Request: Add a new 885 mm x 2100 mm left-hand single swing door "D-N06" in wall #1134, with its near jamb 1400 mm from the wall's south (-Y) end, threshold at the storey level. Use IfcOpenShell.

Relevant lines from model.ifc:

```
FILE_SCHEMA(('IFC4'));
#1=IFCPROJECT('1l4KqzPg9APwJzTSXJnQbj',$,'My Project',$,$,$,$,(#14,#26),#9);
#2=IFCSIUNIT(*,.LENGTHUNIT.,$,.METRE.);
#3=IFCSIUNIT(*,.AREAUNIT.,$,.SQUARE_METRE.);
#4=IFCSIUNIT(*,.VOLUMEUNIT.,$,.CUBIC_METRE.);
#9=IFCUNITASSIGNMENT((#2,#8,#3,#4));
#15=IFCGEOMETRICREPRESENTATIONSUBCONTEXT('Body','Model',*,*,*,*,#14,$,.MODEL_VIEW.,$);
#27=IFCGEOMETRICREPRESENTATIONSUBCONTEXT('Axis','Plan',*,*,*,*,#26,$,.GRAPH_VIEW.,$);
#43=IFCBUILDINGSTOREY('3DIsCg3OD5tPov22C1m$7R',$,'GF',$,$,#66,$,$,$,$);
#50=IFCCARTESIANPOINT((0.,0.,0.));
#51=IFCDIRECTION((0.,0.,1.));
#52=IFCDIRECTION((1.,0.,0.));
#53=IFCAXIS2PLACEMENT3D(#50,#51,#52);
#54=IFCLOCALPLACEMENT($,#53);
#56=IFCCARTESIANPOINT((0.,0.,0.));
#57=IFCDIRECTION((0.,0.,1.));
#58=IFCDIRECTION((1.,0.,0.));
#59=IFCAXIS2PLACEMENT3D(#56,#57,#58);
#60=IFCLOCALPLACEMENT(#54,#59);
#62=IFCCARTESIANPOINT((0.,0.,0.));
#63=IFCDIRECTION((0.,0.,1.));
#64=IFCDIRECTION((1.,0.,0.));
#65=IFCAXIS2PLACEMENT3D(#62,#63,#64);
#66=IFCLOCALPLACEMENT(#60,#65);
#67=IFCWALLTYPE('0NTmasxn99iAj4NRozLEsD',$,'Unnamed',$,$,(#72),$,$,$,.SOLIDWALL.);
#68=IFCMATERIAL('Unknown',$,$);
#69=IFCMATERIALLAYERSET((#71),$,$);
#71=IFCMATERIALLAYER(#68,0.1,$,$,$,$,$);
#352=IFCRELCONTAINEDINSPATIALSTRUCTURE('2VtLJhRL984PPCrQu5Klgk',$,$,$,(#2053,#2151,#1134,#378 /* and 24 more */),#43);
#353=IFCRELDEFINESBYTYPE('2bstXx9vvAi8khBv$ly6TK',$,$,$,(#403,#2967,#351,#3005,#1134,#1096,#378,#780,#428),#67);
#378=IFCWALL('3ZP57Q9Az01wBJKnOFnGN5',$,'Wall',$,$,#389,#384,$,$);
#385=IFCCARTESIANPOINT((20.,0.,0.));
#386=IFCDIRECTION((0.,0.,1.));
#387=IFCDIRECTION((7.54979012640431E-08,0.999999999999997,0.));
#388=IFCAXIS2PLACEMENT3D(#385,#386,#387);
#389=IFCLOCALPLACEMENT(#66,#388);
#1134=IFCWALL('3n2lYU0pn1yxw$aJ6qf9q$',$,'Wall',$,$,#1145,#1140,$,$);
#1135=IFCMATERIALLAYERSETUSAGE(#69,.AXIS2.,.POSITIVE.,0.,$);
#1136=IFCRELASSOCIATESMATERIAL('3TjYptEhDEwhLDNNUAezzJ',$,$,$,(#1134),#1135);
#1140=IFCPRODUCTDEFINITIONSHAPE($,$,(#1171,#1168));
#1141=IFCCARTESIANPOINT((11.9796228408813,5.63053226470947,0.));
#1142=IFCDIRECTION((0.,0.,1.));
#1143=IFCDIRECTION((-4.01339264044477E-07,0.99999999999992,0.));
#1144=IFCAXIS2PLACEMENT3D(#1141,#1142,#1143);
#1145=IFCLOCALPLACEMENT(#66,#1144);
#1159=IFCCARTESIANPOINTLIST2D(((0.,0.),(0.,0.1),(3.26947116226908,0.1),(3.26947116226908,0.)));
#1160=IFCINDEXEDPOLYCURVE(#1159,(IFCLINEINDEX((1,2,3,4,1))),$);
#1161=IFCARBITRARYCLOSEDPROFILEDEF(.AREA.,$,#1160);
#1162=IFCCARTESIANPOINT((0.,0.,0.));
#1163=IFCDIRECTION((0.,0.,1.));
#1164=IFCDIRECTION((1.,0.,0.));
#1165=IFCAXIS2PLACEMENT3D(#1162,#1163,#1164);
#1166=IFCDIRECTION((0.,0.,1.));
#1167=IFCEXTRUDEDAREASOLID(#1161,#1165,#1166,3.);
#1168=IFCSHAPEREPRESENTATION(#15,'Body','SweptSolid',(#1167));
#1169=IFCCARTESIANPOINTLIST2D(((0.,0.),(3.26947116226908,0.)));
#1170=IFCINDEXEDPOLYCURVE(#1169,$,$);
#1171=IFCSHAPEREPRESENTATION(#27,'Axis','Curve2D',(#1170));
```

```python
import numpy as np
import ifcopenshell
import ifcopenshell.api.feature
import ifcopenshell.api.geometry
import ifcopenshell.api.root
import ifcopenshell.api.spatial
import ifcopenshell.geom
import ifcopenshell.util.element
import ifcopenshell.util.placement
import ifcopenshell.util.representation
import ifcopenshell.util.shape
import ifcopenshell.util.unit

model = ifcopenshell.open("model.ifc")
unit_scale = ifcopenshell.util.unit.calculate_unit_scale(model)
settings = ifcopenshell.geom.settings()


def volume(element):
    """Net volume in cubic metres, openings subtracted."""
    shape = ifcopenshell.geom.create_shape(settings, element)
    return ifcopenshell.util.shape.get_volume(shape.geometry)


wall = model.by_guid("3n2lYU0pn1yxw$aJ6qf9q$")
storey = ifcopenshell.util.element.get_container(wall, ifc_class="IfcBuildingStorey")
context = ifcopenshell.util.representation.get_context(model, "Model", "Body", "MODEL_VIEW")
before = volume(wall)

width, height, from_end, sill = 0.885, 2.1, 1.4, 0.0  # metres

# The wall runs along its own X axis, and the end named is its -X end.
wall_shape = ifcopenshell.geom.create_shape(settings, wall)
x, y, z = ifcopenshell.util.shape.get_vertices(wall_shape.geometry).T
start = x.min() + from_end
face, thickness = float(y.min()), float(y.max() - y.min())
wall_matrix = ifcopenshell.util.placement.get_local_placement(wall.ObjectPlacement)
level = ifcopenshell.util.placement.get_local_placement(storey.ObjectPlacement)[2, 3]


def in_wall(x, y):
    """Placement at x, y metres in the wall's axes, at sill height."""
    matrix = wall_matrix.copy()
    matrix[:, 3] = wall_matrix @ np.array([x / unit_scale, y / unit_scale, 0.0, 1.0])
    matrix[2, 3] = level + sill / unit_scale
    return matrix


# Opening: a box that overshoots both wall faces by 50 mm.
opening = ifcopenshell.api.root.create_entity(model, ifc_class="IfcOpeningElement", predefined_type="OPENING")
box = ifcopenshell.api.geometry.add_wall_representation(
    model, context=context, length=width, height=height, thickness=thickness + 0.1
)
ifcopenshell.api.geometry.assign_representation(model, product=opening, representation=box)
ifcopenshell.api.geometry.edit_object_placement(model, product=opening, matrix=in_wall(start, face - 0.05), is_si=False)
ifcopenshell.api.feature.add_feature(model, feature=opening, element=wall)

door = ifcopenshell.api.root.create_entity(model, ifc_class="IfcDoor", name="D-N06", predefined_type="DOOR")
door.OverallWidth, door.OverallHeight = width / unit_scale, height / unit_scale
door.OperationType = "SINGLE_SWING_LEFT"
body = ifcopenshell.api.geometry.add_door_representation(
    model,
    context=context,
    overall_width=door.OverallWidth,
    overall_height=door.OverallHeight,
    operation_type="SINGLE_SWING_LEFT",
    lining_properties={"LiningDepth": thickness / unit_scale, "ThresholdDepth": thickness / unit_scale},
)
ifcopenshell.api.geometry.assign_representation(model, product=door, representation=body)
ifcopenshell.api.spatial.assign_container(model, products=[door], relating_structure=storey)
ifcopenshell.api.feature.add_filling(model, opening=opening, element=door)

# The lining spans the wall, so the door starts at the wall face.
ifcopenshell.api.geometry.edit_object_placement(model, product=door, matrix=in_wall(start, face), is_si=False)

after = volume(wall)

print(f"wall volume {before:.3f} -> {after:.3f} m3")

model.write("model_updated.ifc")
```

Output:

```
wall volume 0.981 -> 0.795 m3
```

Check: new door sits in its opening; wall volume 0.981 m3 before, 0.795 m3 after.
